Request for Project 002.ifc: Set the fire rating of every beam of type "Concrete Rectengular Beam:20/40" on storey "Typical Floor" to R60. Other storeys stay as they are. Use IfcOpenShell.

First a look at what the model holds.

```python
import ifcopenshell
import ifcopenshell.util.element

model = ifcopenshell.open("Project 002.ifc")
print(model.schema)
storey = next(s for s in model.by_type("IfcBuildingStorey") if s.Name == "Typical Floor")
beams = [e for e in ifcopenshell.util.element.get_decomposition(storey) if e.is_a("IfcBeam")]
seen = {}
for e in beams:
    element_type = ifcopenshell.util.element.get_type(e)
    key = (element_type.Name if element_type != e and element_type else None, ifcopenshell.util.element.get_pset(e, "Pset_BeamCommon", "FireRating"))
    seen[key] = seen.get(key, 0) + 1
for (name, value), count in sorted(seen.items(), key=str):
    print(count, "x", name, "|", value)
```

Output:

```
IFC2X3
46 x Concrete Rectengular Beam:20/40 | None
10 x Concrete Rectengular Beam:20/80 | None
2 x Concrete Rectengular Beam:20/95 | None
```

```python
import ifcopenshell
import ifcopenshell.api.pset
import ifcopenshell.util.element

model = ifcopenshell.open("Project 002.ifc")

storey = next(s for s in model.by_type("IfcBuildingStorey") if s.Name == "Typical Floor")
beams = [e for e in ifcopenshell.util.element.get_decomposition(storey) if e.is_a("IfcBeam")]

count = 0
for e in beams:
    element_type = ifcopenshell.util.element.get_type(e)
    if element_type in (None, e) or element_type.Name != "Concrete Rectengular Beam:20/40":
        continue
    # add_pset returns the element's existing set when there is one.
    pset = ifcopenshell.api.pset.add_pset(model, product=e, name="Pset_BeamCommon")
    ifcopenshell.api.pset.edit_pset(model, pset=pset, properties={"FireRating": "R60"})
    count += 1

print(count, "beams updated")

model.write("Project 002_edited.ifc")
```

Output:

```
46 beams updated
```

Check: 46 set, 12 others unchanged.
